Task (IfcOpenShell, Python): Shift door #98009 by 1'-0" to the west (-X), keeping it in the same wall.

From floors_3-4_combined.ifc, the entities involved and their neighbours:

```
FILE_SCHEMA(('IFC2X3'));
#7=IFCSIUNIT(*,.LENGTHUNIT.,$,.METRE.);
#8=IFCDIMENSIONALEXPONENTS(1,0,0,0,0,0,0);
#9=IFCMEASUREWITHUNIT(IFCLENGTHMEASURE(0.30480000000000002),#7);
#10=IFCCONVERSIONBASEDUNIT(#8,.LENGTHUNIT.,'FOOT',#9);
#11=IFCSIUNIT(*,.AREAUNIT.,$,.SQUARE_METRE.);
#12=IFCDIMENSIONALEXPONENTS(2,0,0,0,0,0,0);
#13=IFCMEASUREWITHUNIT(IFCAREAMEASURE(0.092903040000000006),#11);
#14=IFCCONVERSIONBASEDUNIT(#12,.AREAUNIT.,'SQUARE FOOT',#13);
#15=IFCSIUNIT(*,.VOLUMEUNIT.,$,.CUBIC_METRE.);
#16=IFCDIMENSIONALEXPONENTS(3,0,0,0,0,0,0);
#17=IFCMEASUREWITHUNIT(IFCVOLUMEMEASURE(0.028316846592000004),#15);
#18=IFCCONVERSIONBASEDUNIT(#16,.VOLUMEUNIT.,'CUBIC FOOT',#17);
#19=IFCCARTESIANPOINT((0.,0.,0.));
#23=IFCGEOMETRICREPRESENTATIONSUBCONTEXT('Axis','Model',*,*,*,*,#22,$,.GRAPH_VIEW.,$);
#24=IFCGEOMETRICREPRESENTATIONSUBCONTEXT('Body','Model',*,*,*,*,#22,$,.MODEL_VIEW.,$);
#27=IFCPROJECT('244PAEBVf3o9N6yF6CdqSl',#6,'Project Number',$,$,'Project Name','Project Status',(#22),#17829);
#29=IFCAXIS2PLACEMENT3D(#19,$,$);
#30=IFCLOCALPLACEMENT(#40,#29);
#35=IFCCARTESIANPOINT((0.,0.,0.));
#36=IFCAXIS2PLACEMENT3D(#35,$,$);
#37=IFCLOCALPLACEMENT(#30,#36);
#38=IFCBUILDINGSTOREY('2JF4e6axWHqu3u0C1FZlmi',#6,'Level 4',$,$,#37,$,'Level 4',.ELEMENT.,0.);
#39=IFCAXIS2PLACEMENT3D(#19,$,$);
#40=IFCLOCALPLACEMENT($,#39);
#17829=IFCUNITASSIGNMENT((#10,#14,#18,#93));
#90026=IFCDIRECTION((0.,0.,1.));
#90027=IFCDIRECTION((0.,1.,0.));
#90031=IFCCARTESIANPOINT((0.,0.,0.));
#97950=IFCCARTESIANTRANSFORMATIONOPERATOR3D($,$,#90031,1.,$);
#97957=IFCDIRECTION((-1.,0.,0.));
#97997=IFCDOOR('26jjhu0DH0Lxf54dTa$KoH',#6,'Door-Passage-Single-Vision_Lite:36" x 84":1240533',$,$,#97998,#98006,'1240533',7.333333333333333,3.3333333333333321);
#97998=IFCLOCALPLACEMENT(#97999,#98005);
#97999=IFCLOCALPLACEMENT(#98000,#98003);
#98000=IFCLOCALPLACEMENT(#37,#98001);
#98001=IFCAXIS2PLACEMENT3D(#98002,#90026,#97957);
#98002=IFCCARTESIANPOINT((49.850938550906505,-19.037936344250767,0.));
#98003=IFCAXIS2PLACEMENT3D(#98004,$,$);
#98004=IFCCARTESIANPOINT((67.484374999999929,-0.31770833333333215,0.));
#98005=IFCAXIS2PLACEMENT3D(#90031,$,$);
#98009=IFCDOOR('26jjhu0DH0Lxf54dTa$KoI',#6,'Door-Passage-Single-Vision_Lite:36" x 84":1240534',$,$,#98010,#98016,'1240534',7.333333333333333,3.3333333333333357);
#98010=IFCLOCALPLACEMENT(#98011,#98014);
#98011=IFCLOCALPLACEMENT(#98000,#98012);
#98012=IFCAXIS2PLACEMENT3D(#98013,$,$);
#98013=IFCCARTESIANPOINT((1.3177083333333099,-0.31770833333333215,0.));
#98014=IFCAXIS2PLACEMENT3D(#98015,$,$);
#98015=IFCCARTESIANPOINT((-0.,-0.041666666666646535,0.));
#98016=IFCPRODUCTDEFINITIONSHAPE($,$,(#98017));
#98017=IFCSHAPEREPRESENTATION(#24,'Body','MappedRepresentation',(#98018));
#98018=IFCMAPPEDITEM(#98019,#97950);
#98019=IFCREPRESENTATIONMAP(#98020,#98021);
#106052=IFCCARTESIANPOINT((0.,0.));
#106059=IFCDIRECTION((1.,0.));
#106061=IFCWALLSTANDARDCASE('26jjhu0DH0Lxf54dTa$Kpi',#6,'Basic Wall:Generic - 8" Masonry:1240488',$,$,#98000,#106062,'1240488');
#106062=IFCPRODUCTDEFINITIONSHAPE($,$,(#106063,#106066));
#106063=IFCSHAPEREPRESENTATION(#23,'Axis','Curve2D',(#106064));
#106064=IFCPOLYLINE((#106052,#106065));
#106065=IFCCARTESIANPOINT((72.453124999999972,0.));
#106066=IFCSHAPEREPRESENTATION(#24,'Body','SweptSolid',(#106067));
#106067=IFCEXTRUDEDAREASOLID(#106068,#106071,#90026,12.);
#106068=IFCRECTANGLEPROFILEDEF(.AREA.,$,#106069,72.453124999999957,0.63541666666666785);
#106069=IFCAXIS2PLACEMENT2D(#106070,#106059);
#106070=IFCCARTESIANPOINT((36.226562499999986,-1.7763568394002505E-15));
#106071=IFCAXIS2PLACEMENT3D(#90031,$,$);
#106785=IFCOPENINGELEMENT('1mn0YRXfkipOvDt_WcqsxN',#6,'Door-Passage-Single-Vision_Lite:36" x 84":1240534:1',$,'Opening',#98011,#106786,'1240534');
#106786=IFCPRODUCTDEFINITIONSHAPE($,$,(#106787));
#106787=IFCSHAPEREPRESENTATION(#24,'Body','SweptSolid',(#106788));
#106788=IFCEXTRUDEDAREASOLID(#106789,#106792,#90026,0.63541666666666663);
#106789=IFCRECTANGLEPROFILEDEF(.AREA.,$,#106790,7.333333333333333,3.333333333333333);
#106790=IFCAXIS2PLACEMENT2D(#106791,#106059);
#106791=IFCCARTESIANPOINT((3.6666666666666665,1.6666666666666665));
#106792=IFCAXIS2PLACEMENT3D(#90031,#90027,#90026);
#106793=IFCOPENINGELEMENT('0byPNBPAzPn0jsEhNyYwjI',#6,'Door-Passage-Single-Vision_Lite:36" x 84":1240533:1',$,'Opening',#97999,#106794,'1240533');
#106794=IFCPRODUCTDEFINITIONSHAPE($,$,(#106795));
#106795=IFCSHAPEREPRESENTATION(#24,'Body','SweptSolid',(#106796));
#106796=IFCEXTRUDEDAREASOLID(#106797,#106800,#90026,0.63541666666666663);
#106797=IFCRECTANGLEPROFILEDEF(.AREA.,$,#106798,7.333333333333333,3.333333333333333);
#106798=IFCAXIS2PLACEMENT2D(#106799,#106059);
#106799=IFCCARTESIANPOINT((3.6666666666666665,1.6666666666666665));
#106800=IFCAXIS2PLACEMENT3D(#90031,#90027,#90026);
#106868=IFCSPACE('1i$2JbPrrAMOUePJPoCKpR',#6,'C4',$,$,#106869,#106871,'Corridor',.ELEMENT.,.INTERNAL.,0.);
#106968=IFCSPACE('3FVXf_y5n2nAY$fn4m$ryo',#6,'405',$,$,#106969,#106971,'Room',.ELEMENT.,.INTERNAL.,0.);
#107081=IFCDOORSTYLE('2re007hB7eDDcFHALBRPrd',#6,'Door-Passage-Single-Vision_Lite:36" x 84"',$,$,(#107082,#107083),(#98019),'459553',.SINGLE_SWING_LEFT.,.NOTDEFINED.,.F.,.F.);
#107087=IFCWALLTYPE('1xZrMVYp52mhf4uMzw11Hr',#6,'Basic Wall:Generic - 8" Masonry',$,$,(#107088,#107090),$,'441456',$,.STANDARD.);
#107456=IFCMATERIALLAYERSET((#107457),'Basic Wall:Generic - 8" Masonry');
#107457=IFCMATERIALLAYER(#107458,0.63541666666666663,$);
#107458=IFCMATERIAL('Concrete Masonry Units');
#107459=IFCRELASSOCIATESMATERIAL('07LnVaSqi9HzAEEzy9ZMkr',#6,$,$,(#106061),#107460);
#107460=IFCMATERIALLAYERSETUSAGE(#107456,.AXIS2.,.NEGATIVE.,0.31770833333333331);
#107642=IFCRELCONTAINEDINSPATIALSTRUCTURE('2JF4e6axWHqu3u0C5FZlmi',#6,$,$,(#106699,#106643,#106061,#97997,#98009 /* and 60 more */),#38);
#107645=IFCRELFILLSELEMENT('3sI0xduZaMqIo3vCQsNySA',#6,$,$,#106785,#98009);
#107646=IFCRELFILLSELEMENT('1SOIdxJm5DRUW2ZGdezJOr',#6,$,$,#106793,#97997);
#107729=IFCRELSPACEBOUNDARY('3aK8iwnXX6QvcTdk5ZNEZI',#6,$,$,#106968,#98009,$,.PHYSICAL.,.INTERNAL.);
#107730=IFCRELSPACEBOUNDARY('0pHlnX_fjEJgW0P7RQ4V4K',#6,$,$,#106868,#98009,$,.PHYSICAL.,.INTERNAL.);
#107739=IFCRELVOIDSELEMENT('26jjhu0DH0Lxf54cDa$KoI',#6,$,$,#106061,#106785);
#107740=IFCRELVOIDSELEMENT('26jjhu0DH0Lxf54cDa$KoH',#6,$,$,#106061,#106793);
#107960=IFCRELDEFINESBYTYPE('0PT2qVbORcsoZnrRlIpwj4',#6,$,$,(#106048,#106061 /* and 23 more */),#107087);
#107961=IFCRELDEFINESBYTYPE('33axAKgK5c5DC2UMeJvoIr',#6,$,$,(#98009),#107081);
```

```python
import ifcopenshell
import ifcopenshell.api.geometry
import ifcopenshell.util.placement
import ifcopenshell.util.unit

model = ifcopenshell.open("floors_3-4_combined.ifc")
unit_scale = ifcopenshell.util.unit.calculate_unit_scale(model)

door = model.by_id(98009)
opening = door.FillsVoids[0].RelatingOpeningElement
wall = opening.VoidsElements[0].RelatingBuildingElement

wall_matrix = ifcopenshell.util.placement.get_local_placement(wall.ObjectPlacement)
shift = wall_matrix[:3, 0] * 12 * 0.0254 / unit_scale
before = ifcopenshell.util.placement.get_local_placement(door.ObjectPlacement)[:3, 3].copy()

# The door is placed relative to its opening, so it follows when the opening moves.
matrix = ifcopenshell.util.placement.get_local_placement(opening.ObjectPlacement)
matrix[:3, 3] += shift
ifcopenshell.api.geometry.edit_object_placement(
    model, product=opening, matrix=matrix, is_si=False, should_transform_children=True
)

after = ifcopenshell.util.placement.get_local_placement(door.ObjectPlacement)[:3, 3]
print("door moved by", (after - before).round(3) + 0.0)

model.write("floors_3-4_combined-out.ifc")
```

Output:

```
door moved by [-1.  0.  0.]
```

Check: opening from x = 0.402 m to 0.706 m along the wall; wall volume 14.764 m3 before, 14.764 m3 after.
